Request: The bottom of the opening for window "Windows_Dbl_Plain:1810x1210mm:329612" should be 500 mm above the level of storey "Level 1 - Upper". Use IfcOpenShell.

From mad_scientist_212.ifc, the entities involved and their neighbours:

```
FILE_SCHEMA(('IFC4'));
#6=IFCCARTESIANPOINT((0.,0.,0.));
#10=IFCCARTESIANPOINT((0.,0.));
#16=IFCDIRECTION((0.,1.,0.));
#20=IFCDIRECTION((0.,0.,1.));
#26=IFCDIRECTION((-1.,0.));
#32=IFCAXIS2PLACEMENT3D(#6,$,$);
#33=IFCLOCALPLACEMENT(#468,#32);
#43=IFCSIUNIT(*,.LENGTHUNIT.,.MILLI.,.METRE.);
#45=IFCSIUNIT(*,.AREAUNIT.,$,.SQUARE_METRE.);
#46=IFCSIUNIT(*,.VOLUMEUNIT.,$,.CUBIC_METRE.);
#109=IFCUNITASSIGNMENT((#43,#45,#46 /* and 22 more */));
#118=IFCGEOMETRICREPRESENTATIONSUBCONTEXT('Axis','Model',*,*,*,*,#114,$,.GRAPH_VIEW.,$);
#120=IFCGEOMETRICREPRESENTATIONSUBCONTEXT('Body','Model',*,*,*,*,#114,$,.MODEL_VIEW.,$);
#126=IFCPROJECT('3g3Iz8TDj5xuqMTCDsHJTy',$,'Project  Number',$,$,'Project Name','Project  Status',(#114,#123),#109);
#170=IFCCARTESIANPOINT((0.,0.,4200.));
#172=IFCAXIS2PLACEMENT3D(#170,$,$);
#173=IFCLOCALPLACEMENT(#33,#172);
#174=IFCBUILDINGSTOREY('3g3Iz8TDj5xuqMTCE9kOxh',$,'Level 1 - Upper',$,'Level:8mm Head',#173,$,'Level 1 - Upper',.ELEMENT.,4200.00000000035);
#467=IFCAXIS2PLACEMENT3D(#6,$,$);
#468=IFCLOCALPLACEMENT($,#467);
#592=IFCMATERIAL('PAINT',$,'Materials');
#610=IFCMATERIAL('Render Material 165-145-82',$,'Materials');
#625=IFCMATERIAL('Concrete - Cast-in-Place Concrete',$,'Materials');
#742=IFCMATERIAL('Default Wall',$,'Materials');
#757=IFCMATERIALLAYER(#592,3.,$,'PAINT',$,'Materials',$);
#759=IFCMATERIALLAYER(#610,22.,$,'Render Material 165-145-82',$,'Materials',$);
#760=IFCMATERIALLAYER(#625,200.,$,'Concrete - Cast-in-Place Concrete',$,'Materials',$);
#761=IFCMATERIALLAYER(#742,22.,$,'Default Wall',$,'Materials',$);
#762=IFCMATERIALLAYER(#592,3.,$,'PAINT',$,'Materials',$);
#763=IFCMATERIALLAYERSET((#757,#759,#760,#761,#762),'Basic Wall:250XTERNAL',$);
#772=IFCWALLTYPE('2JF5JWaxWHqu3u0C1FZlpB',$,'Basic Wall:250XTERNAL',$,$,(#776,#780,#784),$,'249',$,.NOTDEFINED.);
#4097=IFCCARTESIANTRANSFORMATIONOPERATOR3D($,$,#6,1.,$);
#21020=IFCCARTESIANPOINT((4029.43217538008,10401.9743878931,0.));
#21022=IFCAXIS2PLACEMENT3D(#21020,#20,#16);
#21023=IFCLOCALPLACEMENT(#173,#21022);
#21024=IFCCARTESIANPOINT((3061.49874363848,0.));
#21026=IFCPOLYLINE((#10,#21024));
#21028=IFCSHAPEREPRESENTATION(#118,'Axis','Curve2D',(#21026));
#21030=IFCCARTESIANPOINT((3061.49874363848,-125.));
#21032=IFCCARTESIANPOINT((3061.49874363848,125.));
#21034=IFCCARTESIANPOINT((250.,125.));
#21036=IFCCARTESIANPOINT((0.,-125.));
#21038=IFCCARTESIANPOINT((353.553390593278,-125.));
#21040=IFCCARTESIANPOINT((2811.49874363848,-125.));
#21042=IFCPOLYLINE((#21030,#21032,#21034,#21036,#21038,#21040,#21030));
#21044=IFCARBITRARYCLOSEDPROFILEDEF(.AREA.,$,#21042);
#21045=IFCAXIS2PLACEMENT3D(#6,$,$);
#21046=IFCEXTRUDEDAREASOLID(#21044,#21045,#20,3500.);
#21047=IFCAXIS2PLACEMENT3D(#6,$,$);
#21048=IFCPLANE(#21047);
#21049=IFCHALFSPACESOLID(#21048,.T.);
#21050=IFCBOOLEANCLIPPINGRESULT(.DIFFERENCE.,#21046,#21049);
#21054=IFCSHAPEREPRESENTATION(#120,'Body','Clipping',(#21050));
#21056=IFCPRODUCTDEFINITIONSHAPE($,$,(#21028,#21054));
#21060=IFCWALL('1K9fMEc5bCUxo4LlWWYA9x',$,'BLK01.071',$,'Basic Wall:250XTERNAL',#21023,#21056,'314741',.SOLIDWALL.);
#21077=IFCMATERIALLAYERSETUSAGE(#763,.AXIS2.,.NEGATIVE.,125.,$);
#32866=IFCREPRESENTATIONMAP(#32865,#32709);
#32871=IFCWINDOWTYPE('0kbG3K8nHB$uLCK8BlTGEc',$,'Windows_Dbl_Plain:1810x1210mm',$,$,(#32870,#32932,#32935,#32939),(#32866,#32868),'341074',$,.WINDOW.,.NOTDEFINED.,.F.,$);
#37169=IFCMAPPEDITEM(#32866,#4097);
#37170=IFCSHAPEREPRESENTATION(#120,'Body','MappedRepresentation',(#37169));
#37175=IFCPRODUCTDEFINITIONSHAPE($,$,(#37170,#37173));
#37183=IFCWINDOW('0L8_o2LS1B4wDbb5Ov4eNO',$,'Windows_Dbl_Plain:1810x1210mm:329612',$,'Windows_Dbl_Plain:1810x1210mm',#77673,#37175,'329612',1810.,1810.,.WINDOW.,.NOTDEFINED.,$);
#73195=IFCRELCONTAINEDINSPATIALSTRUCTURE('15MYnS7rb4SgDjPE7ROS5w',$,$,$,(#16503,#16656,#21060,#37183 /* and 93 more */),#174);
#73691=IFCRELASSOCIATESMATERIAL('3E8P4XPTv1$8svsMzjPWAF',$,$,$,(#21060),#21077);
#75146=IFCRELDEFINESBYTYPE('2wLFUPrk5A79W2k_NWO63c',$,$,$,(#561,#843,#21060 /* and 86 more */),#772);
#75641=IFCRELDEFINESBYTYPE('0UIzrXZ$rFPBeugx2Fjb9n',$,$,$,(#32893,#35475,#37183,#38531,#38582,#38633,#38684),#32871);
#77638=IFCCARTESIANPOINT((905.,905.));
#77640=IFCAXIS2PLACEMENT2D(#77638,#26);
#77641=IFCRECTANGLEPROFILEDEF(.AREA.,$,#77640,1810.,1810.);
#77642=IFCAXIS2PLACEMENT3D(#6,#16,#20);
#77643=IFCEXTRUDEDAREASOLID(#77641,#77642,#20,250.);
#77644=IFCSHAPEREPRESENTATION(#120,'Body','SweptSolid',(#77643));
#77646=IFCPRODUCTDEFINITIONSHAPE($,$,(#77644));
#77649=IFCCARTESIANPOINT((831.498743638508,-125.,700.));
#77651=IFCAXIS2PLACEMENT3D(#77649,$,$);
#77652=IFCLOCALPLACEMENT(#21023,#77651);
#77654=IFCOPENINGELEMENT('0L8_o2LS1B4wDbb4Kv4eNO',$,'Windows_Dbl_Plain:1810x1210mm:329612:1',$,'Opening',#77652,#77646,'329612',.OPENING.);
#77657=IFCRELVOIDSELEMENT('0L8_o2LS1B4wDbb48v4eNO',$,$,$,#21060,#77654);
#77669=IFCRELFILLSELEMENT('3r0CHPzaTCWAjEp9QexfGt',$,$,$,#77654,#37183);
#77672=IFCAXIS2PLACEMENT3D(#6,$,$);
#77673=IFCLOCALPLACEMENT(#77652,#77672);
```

```python
import numpy as np
import ifcopenshell
import ifcopenshell.api.geometry
import ifcopenshell.geom
import ifcopenshell.util.element
import ifcopenshell.util.placement
import ifcopenshell.util.shape
import ifcopenshell.util.unit

model = ifcopenshell.open("mad_scientist_212.ifc")
unit_scale = ifcopenshell.util.unit.calculate_unit_scale(model)

window = model.by_guid("0L8_o2LS1B4wDbb5Ov4eNO")
opening = window.FillsVoids[0].RelatingOpeningElement
storey = ifcopenshell.util.element.get_container(window, ifc_class="IfcBuildingStorey")
level = ifcopenshell.util.placement.get_local_placement(storey.ObjectPlacement)[2, 3]

# The opening's origin need not be at the sill, so measure its lowest point.
shape = ifcopenshell.geom.create_shape(ifcopenshell.geom.settings(), opening)
bottom = ifcopenshell.util.shape.get_shape_bottom_elevation(shape, shape.geometry) / unit_scale
dz = level + 0.5 / unit_scale - bottom

shift = np.array([0.0, 0.0, dz])
# The window is placed relative to its opening, so it follows when the opening moves.
matrix = ifcopenshell.util.placement.get_local_placement(opening.ObjectPlacement)
matrix[:3, 3] += shift
ifcopenshell.api.geometry.edit_object_placement(
    model, product=opening, matrix=matrix, is_si=False, should_transform_children=True
)

print(f"moved by {dz * unit_scale:+.3f} m")

model.write("mad_scientist_212-out.ifc")
```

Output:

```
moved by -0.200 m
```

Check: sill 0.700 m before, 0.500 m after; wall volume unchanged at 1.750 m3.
